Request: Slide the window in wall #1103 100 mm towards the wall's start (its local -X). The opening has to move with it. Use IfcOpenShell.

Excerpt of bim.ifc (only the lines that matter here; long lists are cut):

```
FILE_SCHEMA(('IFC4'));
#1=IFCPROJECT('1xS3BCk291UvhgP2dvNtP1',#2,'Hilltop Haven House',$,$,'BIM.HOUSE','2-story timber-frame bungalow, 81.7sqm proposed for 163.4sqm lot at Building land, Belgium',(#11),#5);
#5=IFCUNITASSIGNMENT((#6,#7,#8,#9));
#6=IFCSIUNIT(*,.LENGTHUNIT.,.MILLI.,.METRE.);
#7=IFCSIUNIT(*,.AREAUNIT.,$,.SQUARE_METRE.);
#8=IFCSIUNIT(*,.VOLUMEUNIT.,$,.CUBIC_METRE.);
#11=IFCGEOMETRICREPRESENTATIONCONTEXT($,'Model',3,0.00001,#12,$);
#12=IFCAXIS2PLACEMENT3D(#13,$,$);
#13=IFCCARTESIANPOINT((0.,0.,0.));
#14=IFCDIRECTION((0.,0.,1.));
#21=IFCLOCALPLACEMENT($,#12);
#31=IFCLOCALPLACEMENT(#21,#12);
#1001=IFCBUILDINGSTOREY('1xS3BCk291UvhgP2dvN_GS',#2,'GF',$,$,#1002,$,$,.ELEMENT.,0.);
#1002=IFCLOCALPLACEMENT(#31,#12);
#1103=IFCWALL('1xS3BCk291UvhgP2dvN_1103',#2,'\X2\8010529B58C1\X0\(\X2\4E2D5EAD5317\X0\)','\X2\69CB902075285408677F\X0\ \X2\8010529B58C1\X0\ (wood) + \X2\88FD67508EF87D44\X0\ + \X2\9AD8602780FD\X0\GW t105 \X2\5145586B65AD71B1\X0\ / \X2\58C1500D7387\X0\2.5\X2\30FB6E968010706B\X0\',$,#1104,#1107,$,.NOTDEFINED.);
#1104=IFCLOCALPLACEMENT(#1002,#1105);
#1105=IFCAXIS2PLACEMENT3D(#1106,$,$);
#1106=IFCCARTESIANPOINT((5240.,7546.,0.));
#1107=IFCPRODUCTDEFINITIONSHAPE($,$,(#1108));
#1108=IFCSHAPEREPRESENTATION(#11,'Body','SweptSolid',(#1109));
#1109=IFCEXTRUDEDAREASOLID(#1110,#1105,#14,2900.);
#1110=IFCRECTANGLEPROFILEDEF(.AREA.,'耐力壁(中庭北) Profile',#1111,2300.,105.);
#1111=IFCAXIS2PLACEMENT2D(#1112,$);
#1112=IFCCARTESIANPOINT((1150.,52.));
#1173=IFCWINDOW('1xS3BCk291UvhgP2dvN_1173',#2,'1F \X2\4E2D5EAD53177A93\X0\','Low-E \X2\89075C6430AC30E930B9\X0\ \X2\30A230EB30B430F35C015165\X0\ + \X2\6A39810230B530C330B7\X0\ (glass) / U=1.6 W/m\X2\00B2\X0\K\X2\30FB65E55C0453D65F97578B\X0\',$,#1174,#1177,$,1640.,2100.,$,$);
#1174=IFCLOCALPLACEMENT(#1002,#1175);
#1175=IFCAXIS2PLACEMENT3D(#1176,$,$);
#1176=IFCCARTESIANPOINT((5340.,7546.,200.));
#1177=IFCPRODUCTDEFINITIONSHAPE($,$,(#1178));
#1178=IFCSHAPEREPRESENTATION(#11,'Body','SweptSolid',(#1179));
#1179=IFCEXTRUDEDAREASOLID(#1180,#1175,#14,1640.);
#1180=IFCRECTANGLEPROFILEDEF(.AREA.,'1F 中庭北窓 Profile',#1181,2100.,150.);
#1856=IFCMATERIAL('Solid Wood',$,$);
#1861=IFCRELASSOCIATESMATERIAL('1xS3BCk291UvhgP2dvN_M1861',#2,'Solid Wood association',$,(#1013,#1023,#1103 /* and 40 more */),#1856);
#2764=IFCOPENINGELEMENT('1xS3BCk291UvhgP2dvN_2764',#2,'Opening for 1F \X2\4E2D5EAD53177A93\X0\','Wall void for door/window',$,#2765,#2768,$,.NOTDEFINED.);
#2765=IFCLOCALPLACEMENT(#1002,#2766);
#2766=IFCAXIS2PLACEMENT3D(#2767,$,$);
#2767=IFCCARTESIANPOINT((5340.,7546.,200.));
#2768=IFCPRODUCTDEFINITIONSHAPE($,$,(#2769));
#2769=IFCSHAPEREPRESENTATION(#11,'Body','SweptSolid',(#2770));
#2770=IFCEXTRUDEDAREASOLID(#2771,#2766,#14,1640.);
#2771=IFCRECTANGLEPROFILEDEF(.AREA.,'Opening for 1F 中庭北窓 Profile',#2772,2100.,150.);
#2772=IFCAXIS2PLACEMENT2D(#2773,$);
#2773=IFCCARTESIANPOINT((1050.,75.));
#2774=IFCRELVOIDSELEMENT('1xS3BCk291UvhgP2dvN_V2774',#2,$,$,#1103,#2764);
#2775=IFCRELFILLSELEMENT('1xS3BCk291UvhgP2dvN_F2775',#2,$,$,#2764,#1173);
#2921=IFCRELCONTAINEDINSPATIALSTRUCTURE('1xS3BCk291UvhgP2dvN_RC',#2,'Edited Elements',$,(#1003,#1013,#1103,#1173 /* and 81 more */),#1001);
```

```python
import ifcopenshell
import ifcopenshell.api.geometry
import ifcopenshell.util.placement
import ifcopenshell.util.unit

model = ifcopenshell.open("bim.ifc")
unit_scale = ifcopenshell.util.unit.calculate_unit_scale(model)

window = model.by_id(1173)
opening = window.FillsVoids[0].RelatingOpeningElement
wall = opening.VoidsElements[0].RelatingBuildingElement

wall_matrix = ifcopenshell.util.placement.get_local_placement(wall.ObjectPlacement)
shift = wall_matrix[:3, 0] * -0.1 / unit_scale
before = ifcopenshell.util.placement.get_local_placement(window.ObjectPlacement)[:3, 3].copy()

# The window is not placed relative to its opening, so move both.
for product in (opening, window):
    matrix = ifcopenshell.util.placement.get_local_placement(product.ObjectPlacement)
    matrix[:3, 3] += shift
    ifcopenshell.api.geometry.edit_object_placement(model, product=product, matrix=matrix, is_si=False)

after = ifcopenshell.util.placement.get_local_placement(window.ObjectPlacement)[:3, 3]
print("window moved by", (after - before).round(3) + 0.0)

model.write("bim_v2.ifc")
```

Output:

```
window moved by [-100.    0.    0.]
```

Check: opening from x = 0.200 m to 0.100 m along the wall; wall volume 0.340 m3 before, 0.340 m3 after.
